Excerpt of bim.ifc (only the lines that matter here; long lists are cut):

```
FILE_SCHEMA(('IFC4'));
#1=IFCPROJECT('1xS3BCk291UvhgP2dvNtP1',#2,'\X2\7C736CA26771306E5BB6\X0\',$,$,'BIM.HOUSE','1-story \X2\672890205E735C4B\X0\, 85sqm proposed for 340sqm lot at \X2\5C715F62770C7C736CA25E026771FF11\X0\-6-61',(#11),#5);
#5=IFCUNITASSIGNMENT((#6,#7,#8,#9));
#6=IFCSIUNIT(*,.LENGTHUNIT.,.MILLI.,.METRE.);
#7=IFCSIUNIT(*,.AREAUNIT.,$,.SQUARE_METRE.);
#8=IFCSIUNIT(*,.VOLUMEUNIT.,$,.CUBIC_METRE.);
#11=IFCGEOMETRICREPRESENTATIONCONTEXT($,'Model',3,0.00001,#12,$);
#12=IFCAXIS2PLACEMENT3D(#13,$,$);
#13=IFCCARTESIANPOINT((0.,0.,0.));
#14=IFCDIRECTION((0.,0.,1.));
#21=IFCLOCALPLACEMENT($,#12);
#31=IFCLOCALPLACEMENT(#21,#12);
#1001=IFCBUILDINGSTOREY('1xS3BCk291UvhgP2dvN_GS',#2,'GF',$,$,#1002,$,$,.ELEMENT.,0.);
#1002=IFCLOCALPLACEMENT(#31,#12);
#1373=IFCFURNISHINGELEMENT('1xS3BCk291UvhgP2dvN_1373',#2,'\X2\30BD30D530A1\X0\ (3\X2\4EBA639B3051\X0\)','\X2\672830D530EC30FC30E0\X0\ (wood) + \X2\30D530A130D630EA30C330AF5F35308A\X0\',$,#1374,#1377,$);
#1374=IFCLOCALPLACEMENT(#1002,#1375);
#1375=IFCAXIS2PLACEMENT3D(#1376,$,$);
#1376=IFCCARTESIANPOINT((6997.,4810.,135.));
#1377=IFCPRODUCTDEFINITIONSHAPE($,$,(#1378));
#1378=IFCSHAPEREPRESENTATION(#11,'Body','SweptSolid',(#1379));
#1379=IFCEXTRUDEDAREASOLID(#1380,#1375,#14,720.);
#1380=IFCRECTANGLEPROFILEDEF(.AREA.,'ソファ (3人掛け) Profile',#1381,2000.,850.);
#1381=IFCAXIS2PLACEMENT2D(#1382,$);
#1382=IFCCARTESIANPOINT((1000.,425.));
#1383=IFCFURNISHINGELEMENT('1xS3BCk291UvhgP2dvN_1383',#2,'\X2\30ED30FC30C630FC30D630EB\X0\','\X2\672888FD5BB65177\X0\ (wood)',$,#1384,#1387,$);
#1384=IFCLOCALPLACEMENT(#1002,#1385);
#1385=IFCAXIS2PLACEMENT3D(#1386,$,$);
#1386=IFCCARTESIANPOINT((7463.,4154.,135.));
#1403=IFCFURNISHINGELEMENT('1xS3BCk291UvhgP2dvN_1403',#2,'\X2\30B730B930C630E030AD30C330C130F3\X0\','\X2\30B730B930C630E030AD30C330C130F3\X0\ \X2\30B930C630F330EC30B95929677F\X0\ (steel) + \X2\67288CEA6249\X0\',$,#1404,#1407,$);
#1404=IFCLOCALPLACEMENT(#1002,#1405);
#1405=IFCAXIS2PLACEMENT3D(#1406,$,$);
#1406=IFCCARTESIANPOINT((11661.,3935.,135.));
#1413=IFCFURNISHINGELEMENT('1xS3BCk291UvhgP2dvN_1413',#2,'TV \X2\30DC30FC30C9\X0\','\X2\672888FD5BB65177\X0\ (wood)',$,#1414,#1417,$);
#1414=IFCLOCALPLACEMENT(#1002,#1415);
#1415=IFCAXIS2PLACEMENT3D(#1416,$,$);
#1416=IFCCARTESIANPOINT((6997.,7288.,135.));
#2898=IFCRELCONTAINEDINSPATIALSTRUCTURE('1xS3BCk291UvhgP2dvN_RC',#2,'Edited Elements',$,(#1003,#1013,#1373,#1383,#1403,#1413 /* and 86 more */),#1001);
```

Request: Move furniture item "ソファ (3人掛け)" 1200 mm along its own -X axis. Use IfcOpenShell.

```python
import ifcopenshell
import ifcopenshell.api.geometry
import ifcopenshell.util.placement
import ifcopenshell.util.unit

model = ifcopenshell.open("bim.ifc")
unit_scale = ifcopenshell.util.unit.calculate_unit_scale(model)

item = model.by_guid("1xS3BCk291UvhgP2dvN_1373")
matrix = ifcopenshell.util.placement.get_local_placement(item.ObjectPlacement)
matrix[:3, 3] -= matrix[:3, 0] * 1.2 / unit_scale
ifcopenshell.api.geometry.edit_object_placement(model, product=item, matrix=matrix, is_si=False)

print(ifcopenshell.util.placement.get_local_placement(item.ObjectPlacement).round(3) + 0.0)

model.write("bim-out.ifc")
```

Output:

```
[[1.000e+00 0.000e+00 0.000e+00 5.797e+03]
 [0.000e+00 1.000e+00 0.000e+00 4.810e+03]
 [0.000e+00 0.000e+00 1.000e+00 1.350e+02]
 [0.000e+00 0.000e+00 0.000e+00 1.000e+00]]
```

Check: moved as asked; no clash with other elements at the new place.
